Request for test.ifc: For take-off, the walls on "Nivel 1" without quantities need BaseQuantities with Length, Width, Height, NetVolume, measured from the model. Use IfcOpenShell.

First a look at what the model holds.

```python
import ifcopenshell
import ifcopenshell.util.element
import ifcopenshell.util.unit

model = ifcopenshell.open("test.ifc")
print(model.schema)
for unit_type in ("LENGTHUNIT", "AREAUNIT", "VOLUMEUNIT"):
    print(unit_type, ifcopenshell.util.unit.calculate_unit_scale(model, unit_type))
storey = next(s for s in model.by_type("IfcBuildingStorey") if s.Name == "Nivel 1")
walls = [e for e in ifcopenshell.util.element.get_decomposition(storey) if e.is_a("IfcWall")]
for e in sorted(walls, key=lambda e: e.id()):
    print(e.id(), e.is_a(), e.Name, list(ifcopenshell.util.element.get_psets(e, qtos_only=True)), sep=" | ")
```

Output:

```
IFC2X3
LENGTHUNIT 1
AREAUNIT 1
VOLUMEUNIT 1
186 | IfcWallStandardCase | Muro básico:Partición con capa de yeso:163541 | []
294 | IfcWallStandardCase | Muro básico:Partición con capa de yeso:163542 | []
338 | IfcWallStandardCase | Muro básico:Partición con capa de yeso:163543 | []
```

```python
import ifcopenshell
import ifcopenshell.api.pset
import ifcopenshell.geom
import ifcopenshell.util.element
import ifcopenshell.util.shape
import ifcopenshell.util.unit

model = ifcopenshell.open("test.ifc")
unit_scale = ifcopenshell.util.unit.calculate_unit_scale(model)
volume_scale = ifcopenshell.util.unit.calculate_unit_scale(model, "VOLUMEUNIT")
settings = ifcopenshell.geom.settings()

storey = next(s for s in model.by_type("IfcBuildingStorey") if s.Name == "Nivel 1")
walls = [e for e in ifcopenshell.util.element.get_decomposition(storey) if e.is_a("IfcWall")]

for e in sorted(walls, key=lambda e: e.id()):
    if ifcopenshell.util.element.get_psets(e, qtos_only=True, should_inherit=False):
        continue
    # Geometry comes back in metres, in the element's own axes.
    shape = ifcopenshell.geom.create_shape(settings, e)
    values = {
        "Length": ifcopenshell.util.shape.get_x(shape.geometry) / unit_scale,
        "Width": ifcopenshell.util.shape.get_y(shape.geometry) / unit_scale,
        "Height": ifcopenshell.util.shape.get_z(shape.geometry) / unit_scale,
        "NetVolume": ifcopenshell.util.shape.get_volume(shape.geometry) / volume_scale,
    }
    qto = ifcopenshell.api.pset.add_qto(model, product=e, name="BaseQuantities")
    ifcopenshell.api.pset.edit_qto(model, qto=qto, properties=values)
    print(e.id(), {k: round(v, 3) for k, v in values.items()})

model.write("test-out.ifc")
```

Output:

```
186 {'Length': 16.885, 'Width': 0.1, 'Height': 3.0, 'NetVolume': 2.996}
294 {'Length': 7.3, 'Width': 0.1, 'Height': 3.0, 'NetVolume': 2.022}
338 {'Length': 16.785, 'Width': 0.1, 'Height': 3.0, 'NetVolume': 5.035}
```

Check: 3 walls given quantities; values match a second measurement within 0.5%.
